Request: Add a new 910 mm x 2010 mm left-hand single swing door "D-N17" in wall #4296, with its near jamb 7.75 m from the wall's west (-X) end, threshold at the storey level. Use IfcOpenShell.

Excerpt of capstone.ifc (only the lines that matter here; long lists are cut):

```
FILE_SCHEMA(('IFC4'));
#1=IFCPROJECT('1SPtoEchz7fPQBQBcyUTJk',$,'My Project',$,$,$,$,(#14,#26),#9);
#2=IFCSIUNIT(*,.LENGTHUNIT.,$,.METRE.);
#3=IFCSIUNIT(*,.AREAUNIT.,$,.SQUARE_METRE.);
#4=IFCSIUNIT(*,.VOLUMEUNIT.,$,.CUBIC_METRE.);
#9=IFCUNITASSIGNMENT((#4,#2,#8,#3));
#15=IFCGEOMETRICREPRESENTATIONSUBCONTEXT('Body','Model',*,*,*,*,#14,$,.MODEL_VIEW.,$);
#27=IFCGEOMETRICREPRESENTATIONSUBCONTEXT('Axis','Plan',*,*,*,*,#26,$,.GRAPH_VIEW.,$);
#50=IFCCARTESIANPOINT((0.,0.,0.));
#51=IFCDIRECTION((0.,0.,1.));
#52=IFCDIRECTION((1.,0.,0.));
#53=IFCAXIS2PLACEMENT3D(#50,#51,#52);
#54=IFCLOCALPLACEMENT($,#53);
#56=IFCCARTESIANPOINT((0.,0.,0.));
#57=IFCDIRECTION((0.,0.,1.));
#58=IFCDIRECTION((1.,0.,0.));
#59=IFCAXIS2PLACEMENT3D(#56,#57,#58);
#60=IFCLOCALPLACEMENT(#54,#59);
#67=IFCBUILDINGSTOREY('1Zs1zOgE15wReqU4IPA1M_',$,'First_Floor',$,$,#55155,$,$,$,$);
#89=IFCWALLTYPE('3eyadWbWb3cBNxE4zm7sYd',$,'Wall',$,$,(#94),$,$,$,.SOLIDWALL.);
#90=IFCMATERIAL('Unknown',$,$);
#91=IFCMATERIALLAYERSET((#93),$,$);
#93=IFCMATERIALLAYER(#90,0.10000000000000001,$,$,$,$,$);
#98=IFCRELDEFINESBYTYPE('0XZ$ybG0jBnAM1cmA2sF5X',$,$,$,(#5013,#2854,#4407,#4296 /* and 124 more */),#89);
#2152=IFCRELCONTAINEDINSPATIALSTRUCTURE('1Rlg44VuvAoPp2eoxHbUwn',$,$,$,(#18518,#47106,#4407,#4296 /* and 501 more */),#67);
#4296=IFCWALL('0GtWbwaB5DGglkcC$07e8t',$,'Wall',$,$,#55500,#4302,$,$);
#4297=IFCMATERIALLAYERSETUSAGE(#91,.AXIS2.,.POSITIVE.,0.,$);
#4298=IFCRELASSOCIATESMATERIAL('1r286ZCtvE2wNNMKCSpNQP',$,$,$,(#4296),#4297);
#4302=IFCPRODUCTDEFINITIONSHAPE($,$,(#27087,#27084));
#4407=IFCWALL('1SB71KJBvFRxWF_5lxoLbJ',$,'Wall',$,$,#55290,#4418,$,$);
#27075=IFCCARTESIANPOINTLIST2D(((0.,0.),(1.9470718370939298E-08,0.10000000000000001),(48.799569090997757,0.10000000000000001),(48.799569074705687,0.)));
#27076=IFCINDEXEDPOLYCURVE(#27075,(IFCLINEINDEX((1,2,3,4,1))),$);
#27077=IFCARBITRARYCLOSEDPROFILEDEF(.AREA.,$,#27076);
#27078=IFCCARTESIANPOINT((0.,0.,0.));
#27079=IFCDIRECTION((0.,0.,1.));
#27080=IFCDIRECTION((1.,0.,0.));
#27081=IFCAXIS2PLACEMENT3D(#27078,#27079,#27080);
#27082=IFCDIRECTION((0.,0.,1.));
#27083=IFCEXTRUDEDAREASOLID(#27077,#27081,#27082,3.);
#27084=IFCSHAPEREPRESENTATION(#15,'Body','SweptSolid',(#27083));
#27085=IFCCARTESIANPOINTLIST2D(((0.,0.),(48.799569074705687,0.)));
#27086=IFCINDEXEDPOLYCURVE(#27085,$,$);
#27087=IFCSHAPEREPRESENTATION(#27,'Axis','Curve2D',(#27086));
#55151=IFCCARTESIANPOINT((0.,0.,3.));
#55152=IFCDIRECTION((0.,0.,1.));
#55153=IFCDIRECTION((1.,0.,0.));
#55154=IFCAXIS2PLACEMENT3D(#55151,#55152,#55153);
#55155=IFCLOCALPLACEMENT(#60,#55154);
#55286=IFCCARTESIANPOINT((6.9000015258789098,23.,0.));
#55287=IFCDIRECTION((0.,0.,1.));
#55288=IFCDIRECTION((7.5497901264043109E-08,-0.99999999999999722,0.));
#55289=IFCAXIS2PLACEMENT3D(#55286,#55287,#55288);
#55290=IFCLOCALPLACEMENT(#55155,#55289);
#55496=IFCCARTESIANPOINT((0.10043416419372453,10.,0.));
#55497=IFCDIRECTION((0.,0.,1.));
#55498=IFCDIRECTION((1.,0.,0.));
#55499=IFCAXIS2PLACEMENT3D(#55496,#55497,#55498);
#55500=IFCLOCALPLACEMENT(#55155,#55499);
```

```python
import numpy as np
import ifcopenshell
import ifcopenshell.api.feature
import ifcopenshell.api.geometry
import ifcopenshell.api.root
import ifcopenshell.api.spatial
import ifcopenshell.geom
import ifcopenshell.util.element
import ifcopenshell.util.placement
import ifcopenshell.util.representation
import ifcopenshell.util.shape
import ifcopenshell.util.unit

model = ifcopenshell.open("capstone.ifc")
unit_scale = ifcopenshell.util.unit.calculate_unit_scale(model)
settings = ifcopenshell.geom.settings()


def volume(element):
    """Net volume in cubic metres, openings subtracted."""
    shape = ifcopenshell.geom.create_shape(settings, element)
    return ifcopenshell.util.shape.get_volume(shape.geometry)


wall = model.by_id(4296)
storey = ifcopenshell.util.element.get_container(wall, ifc_class="IfcBuildingStorey")
context = ifcopenshell.util.representation.get_context(model, "Model", "Body", "MODEL_VIEW")
before = volume(wall)

width, height, from_end, sill = 0.91, 2.01, 7.75, 0.0  # metres

# The wall runs along its own X axis, and the end named is its -X end.
wall_shape = ifcopenshell.geom.create_shape(settings, wall)
x, y, z = ifcopenshell.util.shape.get_vertices(wall_shape.geometry).T
start = x.min() + from_end
face, thickness = float(y.min()), float(y.max() - y.min())
wall_matrix = ifcopenshell.util.placement.get_local_placement(wall.ObjectPlacement)
level = ifcopenshell.util.placement.get_local_placement(storey.ObjectPlacement)[2, 3]


def in_wall(x, y):
    """Placement at x, y metres in the wall's axes, at sill height."""
    matrix = wall_matrix.copy()
    matrix[:, 3] = wall_matrix @ np.array([x / unit_scale, y / unit_scale, 0.0, 1.0])
    matrix[2, 3] = level + sill / unit_scale
    return matrix


# Opening: a box that overshoots both wall faces by 50 mm.
opening = ifcopenshell.api.root.create_entity(model, ifc_class="IfcOpeningElement", predefined_type="OPENING")
box = ifcopenshell.api.geometry.add_wall_representation(
    model, context=context, length=width, height=height, thickness=thickness + 0.1
)
ifcopenshell.api.geometry.assign_representation(model, product=opening, representation=box)
ifcopenshell.api.geometry.edit_object_placement(model, product=opening, matrix=in_wall(start, face - 0.05), is_si=False)
ifcopenshell.api.feature.add_feature(model, feature=opening, element=wall)

door = ifcopenshell.api.root.create_entity(model, ifc_class="IfcDoor", name="D-N17", predefined_type="DOOR")
door.OverallWidth, door.OverallHeight = width / unit_scale, height / unit_scale
door.OperationType = "SINGLE_SWING_LEFT"
body = ifcopenshell.api.geometry.add_door_representation(
    model,
    context=context,
    overall_width=door.OverallWidth,
    overall_height=door.OverallHeight,
    operation_type="SINGLE_SWING_LEFT",
    lining_properties={"LiningDepth": thickness / unit_scale, "ThresholdDepth": thickness / unit_scale},
)
ifcopenshell.api.geometry.assign_representation(model, product=door, representation=body)
ifcopenshell.api.spatial.assign_container(model, products=[door], relating_structure=storey)
ifcopenshell.api.feature.add_filling(model, opening=opening, element=door)

# The lining spans the wall, so the door starts at the wall face.
ifcopenshell.api.geometry.edit_object_placement(model, product=door, matrix=in_wall(start, face), is_si=False)

after = volume(wall)

print(f"wall volume {before:.3f} -> {after:.3f} m3")

model.write("capstone_rev.ifc")
```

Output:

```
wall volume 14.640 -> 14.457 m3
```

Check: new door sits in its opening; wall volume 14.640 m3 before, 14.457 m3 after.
